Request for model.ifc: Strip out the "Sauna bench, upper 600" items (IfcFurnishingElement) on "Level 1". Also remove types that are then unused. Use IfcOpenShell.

First a look at what the model holds.

```python
import ifcopenshell
import ifcopenshell.util.element

model = ifcopenshell.open("model.ifc")
print(model.schema)
storey = next(s for s in model.by_type("IfcBuildingStorey") if s.Name == "Level 1")
furniture = [e for e in ifcopenshell.util.element.get_decomposition(storey) if e.is_a("IfcFurnishingElement")]
seen = {}
for e in furniture:
    element_type = ifcopenshell.util.element.get_type(e)
    name = element_type.Name if element_type not in (None, e) else None
    seen[name] = seen.get(name, 0) + 1
for name, count in sorted(seen.items(), key=str):
    print(count, "x", name)
```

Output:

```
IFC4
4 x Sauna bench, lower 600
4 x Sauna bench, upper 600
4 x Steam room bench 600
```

```python
import ifcopenshell
import ifcopenshell.api.root
import ifcopenshell.util.element

model = ifcopenshell.open("model.ifc")

storey = next(s for s in model.by_type("IfcBuildingStorey") if s.Name == "Level 1")
furniture = [e for e in ifcopenshell.util.element.get_decomposition(storey) if e.is_a("IfcFurnishingElement")]
targets = [e for e in furniture if (t := ifcopenshell.util.element.get_type(e)) not in (None, e) and t.Name == "Sauna bench, upper 600"]
types = {ifcopenshell.util.element.get_type(e) for e in targets} - {None, *targets}

for e in targets:
    ifcopenshell.api.root.remove_product(model, product=e)
print(len(targets), "removed")

unused = [t for t in types if not ifcopenshell.util.element.get_types(t)]
for t in unused:
    ifcopenshell.api.root.remove_product(model, product=t)
print(len(unused), "unused types removed")

model.write("model_edited.ifc")
```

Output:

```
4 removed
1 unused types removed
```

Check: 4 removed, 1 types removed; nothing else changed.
